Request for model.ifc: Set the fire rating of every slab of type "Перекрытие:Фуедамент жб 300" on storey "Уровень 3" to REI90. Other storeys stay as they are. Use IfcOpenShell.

First a look at what the model holds.

```python
import ifcopenshell
import ifcopenshell.util.element

model = ifcopenshell.open("model.ifc")
print(model.schema)
storey = next(s for s in model.by_type("IfcBuildingStorey") if s.Name == "Уровень 3")
slabs = [e for e in ifcopenshell.util.element.get_decomposition(storey) if e.is_a("IfcSlab")]
seen = {}
for e in slabs:
    element_type = ifcopenshell.util.element.get_type(e)
    key = (element_type.Name if element_type != e and element_type else None, ifcopenshell.util.element.get_pset(e, "Pset_SlabCommon", "FireRating"))
    seen[key] = seen.get(key, 0) + 1
for (name, value), count in sorted(seen.items(), key=str):
    print(count, "x", name, "|", value)
```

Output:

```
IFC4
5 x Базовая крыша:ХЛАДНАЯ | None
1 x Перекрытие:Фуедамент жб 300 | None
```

```python
import ifcopenshell
import ifcopenshell.api.pset
import ifcopenshell.util.element

model = ifcopenshell.open("model.ifc")

storey = next(s for s in model.by_type("IfcBuildingStorey") if s.Name == "Уровень 3")
slabs = [e for e in ifcopenshell.util.element.get_decomposition(storey) if e.is_a("IfcSlab")]

count = 0
for e in slabs:
    element_type = ifcopenshell.util.element.get_type(e)
    if element_type in (None, e) or element_type.Name != "Перекрытие:Фуедамент жб 300":
        continue
    # add_pset returns the element's existing set when there is one.
    pset = ifcopenshell.api.pset.add_pset(model, product=e, name="Pset_SlabCommon")
    ifcopenshell.api.pset.edit_pset(model, pset=pset, properties={"FireRating": "REI90"})
    count += 1

print(count, "slabs updated")

model.write("model_updated.ifc")
```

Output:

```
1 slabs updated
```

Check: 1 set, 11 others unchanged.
